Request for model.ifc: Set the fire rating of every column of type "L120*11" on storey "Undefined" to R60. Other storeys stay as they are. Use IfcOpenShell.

First a look at what the model holds.

```python
import ifcopenshell
import ifcopenshell.util.element

model = ifcopenshell.open("model.ifc")
print(model.schema)
storey = next(s for s in model.by_type("IfcBuildingStorey") if s.Name == "Undefined")
columns = [e for e in ifcopenshell.util.element.get_decomposition(storey) if e.is_a("IfcColumn")]
seen = {}
for e in columns:
    element_type = ifcopenshell.util.element.get_type(e)
    key = (element_type.Name if element_type != e and element_type else None, ifcopenshell.util.element.get_pset(e, "Pset_ColumnCommon", "FireRating"))
    seen[key] = seen.get(key, 0) + 1
for (name, value), count in sorted(seen.items(), key=str):
    print(count, "x", name, "|", value)
```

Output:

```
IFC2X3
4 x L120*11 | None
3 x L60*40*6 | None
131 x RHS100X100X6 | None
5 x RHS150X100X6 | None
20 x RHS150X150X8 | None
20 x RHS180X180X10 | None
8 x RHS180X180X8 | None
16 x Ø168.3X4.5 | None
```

```python
import ifcopenshell
import ifcopenshell.api.pset
import ifcopenshell.util.element

model = ifcopenshell.open("model.ifc")

storey = next(s for s in model.by_type("IfcBuildingStorey") if s.Name == "Undefined")
columns = [e for e in ifcopenshell.util.element.get_decomposition(storey) if e.is_a("IfcColumn")]

count = 0
for e in columns:
    element_type = ifcopenshell.util.element.get_type(e)
    if element_type in (None, e) or element_type.Name != "L120*11":
        continue
    found = ifcopenshell.util.element.get_pset(e, "Pset_ColumnCommon", should_inherit=False)
    if found:
        pset = model.by_id(found["id"])
        if len(ifcopenshell.util.element.get_elements_by_pset(pset)) > 1:
            pset = ifcopenshell.api.pset.unshare_pset(model, products=[e], pset=pset)[0]
    else:
        pset = ifcopenshell.api.pset.add_pset(model, product=e, name="Pset_ColumnCommon")
    ifcopenshell.api.pset.edit_pset(model, pset=pset, properties={"FireRating": "R60"})
    count += 1

print(count, "columns updated")

model.write("model_v2.ifc")
```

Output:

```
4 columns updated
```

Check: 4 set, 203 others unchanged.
